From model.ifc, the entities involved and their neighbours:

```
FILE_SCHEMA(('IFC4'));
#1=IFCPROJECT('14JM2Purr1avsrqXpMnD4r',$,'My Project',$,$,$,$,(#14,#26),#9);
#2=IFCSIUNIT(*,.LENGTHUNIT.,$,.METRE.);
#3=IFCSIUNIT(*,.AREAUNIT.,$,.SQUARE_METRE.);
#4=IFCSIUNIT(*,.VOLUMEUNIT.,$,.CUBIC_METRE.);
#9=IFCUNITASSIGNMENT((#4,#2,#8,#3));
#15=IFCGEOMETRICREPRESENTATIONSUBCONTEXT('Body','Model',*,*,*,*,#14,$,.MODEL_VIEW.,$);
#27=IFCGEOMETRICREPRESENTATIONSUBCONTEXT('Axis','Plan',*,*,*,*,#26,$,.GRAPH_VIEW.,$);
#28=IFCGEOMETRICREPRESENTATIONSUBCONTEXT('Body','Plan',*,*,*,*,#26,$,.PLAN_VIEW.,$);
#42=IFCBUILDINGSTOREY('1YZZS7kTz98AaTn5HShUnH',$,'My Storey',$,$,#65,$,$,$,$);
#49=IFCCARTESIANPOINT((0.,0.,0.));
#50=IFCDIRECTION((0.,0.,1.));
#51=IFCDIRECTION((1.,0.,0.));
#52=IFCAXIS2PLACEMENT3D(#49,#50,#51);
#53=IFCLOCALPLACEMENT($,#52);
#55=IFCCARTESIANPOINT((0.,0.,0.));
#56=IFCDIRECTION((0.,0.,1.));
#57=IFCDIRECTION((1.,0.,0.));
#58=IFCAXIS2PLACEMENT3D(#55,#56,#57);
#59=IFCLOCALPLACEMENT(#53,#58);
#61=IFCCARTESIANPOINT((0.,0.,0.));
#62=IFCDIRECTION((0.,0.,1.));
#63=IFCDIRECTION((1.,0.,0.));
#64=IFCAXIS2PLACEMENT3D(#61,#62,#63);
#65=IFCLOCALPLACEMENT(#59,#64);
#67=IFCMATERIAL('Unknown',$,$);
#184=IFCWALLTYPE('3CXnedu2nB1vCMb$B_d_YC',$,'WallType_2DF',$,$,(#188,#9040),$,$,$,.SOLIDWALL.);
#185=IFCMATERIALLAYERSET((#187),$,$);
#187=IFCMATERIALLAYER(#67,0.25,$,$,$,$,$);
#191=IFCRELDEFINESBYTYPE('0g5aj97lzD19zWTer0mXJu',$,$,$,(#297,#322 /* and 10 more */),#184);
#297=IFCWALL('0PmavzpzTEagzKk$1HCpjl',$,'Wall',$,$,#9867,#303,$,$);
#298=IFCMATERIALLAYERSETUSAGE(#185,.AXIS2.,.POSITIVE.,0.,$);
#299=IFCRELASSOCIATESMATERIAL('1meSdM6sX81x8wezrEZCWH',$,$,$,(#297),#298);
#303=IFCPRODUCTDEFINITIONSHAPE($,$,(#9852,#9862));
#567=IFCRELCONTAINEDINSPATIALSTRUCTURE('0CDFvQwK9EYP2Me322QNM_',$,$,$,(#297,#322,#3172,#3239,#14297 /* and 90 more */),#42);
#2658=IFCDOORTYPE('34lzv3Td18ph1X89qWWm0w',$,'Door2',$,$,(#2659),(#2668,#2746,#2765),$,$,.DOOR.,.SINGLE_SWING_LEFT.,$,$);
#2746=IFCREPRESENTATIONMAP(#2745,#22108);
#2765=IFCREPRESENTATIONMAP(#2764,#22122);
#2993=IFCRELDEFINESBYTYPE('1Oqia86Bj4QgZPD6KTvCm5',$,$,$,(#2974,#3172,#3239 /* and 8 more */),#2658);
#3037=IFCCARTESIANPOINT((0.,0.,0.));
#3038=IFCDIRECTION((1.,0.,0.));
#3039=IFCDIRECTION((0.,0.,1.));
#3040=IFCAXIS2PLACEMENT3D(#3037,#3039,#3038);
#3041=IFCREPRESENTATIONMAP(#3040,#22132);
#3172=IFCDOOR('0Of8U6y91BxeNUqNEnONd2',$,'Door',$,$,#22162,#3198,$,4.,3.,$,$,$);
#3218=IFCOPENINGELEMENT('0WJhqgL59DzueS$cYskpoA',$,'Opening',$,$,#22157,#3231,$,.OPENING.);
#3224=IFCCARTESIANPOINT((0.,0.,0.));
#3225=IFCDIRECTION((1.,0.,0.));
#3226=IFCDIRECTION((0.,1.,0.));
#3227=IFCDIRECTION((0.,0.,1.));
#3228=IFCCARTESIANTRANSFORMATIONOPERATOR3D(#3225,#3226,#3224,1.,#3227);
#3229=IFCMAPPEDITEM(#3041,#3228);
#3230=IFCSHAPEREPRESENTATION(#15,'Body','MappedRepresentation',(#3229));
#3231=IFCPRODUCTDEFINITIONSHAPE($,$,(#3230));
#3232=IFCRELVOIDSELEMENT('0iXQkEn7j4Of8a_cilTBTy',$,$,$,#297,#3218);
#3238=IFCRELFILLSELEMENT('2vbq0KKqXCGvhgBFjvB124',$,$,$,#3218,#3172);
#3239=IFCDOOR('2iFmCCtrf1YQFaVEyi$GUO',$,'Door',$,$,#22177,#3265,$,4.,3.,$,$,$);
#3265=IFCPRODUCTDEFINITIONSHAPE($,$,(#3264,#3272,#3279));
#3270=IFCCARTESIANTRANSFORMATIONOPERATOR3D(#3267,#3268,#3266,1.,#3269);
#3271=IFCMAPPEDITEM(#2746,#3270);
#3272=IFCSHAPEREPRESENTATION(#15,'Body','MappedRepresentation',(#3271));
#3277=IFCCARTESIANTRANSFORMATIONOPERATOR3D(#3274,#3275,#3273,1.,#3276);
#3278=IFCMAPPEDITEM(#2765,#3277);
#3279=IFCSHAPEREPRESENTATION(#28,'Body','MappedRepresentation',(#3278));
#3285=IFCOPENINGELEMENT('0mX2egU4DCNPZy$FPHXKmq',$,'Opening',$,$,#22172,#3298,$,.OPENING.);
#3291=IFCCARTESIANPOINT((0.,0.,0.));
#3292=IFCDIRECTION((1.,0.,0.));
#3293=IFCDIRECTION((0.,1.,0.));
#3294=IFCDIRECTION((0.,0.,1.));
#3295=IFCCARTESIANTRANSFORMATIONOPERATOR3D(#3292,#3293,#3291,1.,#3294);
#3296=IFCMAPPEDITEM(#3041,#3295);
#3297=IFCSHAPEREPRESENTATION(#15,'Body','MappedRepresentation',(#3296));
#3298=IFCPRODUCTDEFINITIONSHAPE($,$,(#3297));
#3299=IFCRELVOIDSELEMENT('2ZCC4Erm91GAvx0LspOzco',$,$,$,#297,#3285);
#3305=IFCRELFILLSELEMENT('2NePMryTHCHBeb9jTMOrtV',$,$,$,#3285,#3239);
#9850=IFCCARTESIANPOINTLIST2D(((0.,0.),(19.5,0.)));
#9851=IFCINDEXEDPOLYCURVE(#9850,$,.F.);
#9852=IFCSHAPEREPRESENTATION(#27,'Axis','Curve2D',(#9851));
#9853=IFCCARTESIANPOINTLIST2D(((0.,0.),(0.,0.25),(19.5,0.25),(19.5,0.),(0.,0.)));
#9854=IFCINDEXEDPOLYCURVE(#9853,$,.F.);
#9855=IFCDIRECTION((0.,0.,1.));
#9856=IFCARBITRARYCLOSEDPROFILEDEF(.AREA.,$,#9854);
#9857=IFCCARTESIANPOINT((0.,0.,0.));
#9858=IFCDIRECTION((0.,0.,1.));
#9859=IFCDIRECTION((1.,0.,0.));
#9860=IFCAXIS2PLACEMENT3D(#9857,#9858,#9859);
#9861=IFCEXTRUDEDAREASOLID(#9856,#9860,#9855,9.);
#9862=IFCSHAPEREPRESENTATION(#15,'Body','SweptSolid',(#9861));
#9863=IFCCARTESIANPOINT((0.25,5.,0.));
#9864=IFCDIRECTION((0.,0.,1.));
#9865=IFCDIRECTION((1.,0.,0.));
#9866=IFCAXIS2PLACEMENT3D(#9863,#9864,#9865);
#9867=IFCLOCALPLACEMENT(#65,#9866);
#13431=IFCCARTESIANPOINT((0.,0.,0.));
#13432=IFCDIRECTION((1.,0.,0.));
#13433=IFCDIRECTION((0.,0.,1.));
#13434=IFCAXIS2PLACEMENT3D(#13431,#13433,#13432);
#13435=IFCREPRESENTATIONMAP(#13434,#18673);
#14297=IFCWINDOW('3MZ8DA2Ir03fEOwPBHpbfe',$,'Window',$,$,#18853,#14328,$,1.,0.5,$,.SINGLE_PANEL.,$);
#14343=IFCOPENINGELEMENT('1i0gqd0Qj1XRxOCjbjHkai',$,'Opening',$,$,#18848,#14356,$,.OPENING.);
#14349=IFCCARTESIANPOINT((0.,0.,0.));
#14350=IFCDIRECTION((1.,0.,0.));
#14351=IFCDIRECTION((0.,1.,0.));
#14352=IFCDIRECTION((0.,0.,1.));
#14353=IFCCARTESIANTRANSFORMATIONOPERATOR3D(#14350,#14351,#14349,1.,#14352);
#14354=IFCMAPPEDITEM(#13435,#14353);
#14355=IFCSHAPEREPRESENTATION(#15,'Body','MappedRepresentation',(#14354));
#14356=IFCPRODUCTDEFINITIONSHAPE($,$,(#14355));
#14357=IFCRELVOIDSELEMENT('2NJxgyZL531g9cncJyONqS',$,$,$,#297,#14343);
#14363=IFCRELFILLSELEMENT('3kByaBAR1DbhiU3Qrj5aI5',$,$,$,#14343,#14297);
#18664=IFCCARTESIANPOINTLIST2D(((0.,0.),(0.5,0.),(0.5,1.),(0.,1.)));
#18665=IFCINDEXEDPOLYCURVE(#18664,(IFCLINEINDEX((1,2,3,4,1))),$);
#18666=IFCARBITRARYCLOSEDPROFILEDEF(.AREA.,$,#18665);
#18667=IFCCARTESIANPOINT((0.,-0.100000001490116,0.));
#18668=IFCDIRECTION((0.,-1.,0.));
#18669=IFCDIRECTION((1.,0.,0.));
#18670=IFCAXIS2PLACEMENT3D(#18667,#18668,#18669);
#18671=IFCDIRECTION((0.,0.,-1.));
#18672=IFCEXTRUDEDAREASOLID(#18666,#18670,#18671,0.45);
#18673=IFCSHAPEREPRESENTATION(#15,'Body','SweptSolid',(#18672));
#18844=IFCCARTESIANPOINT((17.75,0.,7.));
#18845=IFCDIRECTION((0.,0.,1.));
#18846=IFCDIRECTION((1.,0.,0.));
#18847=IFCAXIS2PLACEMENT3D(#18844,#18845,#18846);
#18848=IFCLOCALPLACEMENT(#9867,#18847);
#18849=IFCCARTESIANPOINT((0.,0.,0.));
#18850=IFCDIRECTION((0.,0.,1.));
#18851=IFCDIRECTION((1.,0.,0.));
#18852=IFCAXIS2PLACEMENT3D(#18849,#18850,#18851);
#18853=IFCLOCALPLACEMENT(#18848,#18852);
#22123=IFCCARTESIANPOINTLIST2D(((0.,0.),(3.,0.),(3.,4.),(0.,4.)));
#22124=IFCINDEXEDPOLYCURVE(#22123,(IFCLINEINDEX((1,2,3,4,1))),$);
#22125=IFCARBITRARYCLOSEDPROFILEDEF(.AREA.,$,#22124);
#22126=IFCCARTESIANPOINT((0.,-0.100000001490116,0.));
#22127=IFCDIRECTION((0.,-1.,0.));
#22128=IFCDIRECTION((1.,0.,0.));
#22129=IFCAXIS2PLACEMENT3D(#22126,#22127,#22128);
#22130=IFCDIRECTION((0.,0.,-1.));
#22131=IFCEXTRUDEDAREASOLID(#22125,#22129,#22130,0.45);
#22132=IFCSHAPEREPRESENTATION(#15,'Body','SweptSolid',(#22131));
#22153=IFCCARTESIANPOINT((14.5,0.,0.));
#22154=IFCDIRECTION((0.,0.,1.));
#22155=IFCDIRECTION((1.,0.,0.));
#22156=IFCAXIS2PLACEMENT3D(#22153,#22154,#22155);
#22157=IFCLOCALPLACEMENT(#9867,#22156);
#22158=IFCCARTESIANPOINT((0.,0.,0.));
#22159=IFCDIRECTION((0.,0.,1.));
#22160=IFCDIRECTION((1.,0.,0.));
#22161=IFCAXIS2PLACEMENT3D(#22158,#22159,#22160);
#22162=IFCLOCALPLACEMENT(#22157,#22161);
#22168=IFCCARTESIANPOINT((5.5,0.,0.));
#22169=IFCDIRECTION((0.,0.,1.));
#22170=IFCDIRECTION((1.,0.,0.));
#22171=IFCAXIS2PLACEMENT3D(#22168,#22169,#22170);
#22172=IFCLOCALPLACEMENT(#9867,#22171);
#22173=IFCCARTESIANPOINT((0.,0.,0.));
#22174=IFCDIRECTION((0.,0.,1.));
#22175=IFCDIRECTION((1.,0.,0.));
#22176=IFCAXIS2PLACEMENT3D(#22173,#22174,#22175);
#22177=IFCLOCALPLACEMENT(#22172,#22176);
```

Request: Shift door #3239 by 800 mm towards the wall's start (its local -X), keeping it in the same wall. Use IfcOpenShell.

```python
import ifcopenshell
import ifcopenshell.api.geometry
import ifcopenshell.util.placement

model = ifcopenshell.open("model.ifc")

door = model.by_guid("2iFmCCtrf1YQFaVEyi$GUO")
opening = door.FillsVoids[0].RelatingOpeningElement
wall = opening.VoidsElements[0].RelatingBuildingElement

wall_matrix = ifcopenshell.util.placement.get_local_placement(wall.ObjectPlacement)
shift = wall_matrix[:3, 0] * -0.8
before = ifcopenshell.util.placement.get_local_placement(door.ObjectPlacement)[:3, 3].copy()

# The door is placed relative to its opening, so it follows when the opening moves.
matrix = ifcopenshell.util.placement.get_local_placement(opening.ObjectPlacement)
matrix[:3, 3] += shift
ifcopenshell.api.geometry.edit_object_placement(
    model, product=opening, matrix=matrix, is_si=False, should_transform_children=True
)

after = ifcopenshell.util.placement.get_local_placement(door.ObjectPlacement)[:3, 3]
print("door moved by", (after - before).round(3) + 0.0)

model.write("model-out.ifc")
```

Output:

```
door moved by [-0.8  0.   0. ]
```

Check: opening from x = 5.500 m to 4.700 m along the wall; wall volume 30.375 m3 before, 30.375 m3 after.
